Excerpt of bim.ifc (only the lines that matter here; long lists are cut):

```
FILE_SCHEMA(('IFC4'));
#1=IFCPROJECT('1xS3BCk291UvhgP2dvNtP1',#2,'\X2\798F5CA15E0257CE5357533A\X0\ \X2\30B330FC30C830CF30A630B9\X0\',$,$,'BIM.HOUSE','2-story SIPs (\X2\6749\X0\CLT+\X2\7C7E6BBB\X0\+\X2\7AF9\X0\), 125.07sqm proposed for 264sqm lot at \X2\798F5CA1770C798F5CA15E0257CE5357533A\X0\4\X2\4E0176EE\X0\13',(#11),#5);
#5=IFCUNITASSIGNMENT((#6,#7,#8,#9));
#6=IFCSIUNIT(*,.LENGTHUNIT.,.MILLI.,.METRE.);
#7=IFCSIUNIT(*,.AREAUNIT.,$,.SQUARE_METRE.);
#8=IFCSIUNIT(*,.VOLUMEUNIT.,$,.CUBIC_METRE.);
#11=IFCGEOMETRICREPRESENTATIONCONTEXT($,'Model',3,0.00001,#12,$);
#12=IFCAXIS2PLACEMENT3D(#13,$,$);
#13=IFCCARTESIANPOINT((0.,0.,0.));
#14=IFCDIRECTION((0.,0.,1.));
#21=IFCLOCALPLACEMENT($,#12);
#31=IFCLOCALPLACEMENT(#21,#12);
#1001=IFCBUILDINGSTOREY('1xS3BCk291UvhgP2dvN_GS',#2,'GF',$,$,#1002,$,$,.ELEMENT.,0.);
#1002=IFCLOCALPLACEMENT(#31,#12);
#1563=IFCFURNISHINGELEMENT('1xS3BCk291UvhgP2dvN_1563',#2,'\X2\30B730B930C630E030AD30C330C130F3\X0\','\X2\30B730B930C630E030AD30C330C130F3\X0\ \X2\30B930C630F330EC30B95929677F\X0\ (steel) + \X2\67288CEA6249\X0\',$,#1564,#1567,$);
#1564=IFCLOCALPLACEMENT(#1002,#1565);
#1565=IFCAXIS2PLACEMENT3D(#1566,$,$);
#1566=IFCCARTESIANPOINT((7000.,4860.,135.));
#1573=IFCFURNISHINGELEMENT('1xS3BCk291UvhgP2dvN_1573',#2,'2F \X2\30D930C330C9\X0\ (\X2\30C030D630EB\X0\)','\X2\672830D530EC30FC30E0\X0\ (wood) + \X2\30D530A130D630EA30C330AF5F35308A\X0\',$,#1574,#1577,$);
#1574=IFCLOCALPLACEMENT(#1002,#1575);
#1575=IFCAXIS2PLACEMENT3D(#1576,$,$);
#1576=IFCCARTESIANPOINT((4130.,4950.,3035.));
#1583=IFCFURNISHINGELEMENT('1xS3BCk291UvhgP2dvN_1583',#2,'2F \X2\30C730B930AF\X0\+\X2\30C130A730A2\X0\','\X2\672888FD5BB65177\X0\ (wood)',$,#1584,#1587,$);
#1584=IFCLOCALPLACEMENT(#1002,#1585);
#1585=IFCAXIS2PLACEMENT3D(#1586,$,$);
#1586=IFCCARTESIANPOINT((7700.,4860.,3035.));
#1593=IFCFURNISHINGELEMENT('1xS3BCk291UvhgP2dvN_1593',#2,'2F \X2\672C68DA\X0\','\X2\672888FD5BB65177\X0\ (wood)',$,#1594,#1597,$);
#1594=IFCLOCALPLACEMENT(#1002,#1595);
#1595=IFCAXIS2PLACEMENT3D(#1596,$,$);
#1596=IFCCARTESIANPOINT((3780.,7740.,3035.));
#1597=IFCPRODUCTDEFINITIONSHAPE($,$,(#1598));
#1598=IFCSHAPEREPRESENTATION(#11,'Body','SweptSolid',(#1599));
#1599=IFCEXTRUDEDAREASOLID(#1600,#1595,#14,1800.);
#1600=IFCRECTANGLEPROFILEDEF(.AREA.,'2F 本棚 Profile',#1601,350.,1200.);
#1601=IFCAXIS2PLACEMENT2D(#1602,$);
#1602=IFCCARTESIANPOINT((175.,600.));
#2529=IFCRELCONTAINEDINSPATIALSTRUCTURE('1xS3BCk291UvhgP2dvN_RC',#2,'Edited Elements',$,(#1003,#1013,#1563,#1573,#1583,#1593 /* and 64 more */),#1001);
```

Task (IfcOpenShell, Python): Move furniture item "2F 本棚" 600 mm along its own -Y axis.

```python
import ifcopenshell
import ifcopenshell.api.geometry
import ifcopenshell.util.placement

model = ifcopenshell.open("bim.ifc")

item = model.by_id(1593)
matrix = ifcopenshell.util.placement.get_local_placement(item.ObjectPlacement)
matrix[:3, 3] -= matrix[:3, 1] * 600.0
ifcopenshell.api.geometry.edit_object_placement(model, product=item, matrix=matrix, is_si=False)

print(ifcopenshell.util.placement.get_local_placement(item.ObjectPlacement).round(3) + 0.0)

model.write("bim_updated.ifc")
```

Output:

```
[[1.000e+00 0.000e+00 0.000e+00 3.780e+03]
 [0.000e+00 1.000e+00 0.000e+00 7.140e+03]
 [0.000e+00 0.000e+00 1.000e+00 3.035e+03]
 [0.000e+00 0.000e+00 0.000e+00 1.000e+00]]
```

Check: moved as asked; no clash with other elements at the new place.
